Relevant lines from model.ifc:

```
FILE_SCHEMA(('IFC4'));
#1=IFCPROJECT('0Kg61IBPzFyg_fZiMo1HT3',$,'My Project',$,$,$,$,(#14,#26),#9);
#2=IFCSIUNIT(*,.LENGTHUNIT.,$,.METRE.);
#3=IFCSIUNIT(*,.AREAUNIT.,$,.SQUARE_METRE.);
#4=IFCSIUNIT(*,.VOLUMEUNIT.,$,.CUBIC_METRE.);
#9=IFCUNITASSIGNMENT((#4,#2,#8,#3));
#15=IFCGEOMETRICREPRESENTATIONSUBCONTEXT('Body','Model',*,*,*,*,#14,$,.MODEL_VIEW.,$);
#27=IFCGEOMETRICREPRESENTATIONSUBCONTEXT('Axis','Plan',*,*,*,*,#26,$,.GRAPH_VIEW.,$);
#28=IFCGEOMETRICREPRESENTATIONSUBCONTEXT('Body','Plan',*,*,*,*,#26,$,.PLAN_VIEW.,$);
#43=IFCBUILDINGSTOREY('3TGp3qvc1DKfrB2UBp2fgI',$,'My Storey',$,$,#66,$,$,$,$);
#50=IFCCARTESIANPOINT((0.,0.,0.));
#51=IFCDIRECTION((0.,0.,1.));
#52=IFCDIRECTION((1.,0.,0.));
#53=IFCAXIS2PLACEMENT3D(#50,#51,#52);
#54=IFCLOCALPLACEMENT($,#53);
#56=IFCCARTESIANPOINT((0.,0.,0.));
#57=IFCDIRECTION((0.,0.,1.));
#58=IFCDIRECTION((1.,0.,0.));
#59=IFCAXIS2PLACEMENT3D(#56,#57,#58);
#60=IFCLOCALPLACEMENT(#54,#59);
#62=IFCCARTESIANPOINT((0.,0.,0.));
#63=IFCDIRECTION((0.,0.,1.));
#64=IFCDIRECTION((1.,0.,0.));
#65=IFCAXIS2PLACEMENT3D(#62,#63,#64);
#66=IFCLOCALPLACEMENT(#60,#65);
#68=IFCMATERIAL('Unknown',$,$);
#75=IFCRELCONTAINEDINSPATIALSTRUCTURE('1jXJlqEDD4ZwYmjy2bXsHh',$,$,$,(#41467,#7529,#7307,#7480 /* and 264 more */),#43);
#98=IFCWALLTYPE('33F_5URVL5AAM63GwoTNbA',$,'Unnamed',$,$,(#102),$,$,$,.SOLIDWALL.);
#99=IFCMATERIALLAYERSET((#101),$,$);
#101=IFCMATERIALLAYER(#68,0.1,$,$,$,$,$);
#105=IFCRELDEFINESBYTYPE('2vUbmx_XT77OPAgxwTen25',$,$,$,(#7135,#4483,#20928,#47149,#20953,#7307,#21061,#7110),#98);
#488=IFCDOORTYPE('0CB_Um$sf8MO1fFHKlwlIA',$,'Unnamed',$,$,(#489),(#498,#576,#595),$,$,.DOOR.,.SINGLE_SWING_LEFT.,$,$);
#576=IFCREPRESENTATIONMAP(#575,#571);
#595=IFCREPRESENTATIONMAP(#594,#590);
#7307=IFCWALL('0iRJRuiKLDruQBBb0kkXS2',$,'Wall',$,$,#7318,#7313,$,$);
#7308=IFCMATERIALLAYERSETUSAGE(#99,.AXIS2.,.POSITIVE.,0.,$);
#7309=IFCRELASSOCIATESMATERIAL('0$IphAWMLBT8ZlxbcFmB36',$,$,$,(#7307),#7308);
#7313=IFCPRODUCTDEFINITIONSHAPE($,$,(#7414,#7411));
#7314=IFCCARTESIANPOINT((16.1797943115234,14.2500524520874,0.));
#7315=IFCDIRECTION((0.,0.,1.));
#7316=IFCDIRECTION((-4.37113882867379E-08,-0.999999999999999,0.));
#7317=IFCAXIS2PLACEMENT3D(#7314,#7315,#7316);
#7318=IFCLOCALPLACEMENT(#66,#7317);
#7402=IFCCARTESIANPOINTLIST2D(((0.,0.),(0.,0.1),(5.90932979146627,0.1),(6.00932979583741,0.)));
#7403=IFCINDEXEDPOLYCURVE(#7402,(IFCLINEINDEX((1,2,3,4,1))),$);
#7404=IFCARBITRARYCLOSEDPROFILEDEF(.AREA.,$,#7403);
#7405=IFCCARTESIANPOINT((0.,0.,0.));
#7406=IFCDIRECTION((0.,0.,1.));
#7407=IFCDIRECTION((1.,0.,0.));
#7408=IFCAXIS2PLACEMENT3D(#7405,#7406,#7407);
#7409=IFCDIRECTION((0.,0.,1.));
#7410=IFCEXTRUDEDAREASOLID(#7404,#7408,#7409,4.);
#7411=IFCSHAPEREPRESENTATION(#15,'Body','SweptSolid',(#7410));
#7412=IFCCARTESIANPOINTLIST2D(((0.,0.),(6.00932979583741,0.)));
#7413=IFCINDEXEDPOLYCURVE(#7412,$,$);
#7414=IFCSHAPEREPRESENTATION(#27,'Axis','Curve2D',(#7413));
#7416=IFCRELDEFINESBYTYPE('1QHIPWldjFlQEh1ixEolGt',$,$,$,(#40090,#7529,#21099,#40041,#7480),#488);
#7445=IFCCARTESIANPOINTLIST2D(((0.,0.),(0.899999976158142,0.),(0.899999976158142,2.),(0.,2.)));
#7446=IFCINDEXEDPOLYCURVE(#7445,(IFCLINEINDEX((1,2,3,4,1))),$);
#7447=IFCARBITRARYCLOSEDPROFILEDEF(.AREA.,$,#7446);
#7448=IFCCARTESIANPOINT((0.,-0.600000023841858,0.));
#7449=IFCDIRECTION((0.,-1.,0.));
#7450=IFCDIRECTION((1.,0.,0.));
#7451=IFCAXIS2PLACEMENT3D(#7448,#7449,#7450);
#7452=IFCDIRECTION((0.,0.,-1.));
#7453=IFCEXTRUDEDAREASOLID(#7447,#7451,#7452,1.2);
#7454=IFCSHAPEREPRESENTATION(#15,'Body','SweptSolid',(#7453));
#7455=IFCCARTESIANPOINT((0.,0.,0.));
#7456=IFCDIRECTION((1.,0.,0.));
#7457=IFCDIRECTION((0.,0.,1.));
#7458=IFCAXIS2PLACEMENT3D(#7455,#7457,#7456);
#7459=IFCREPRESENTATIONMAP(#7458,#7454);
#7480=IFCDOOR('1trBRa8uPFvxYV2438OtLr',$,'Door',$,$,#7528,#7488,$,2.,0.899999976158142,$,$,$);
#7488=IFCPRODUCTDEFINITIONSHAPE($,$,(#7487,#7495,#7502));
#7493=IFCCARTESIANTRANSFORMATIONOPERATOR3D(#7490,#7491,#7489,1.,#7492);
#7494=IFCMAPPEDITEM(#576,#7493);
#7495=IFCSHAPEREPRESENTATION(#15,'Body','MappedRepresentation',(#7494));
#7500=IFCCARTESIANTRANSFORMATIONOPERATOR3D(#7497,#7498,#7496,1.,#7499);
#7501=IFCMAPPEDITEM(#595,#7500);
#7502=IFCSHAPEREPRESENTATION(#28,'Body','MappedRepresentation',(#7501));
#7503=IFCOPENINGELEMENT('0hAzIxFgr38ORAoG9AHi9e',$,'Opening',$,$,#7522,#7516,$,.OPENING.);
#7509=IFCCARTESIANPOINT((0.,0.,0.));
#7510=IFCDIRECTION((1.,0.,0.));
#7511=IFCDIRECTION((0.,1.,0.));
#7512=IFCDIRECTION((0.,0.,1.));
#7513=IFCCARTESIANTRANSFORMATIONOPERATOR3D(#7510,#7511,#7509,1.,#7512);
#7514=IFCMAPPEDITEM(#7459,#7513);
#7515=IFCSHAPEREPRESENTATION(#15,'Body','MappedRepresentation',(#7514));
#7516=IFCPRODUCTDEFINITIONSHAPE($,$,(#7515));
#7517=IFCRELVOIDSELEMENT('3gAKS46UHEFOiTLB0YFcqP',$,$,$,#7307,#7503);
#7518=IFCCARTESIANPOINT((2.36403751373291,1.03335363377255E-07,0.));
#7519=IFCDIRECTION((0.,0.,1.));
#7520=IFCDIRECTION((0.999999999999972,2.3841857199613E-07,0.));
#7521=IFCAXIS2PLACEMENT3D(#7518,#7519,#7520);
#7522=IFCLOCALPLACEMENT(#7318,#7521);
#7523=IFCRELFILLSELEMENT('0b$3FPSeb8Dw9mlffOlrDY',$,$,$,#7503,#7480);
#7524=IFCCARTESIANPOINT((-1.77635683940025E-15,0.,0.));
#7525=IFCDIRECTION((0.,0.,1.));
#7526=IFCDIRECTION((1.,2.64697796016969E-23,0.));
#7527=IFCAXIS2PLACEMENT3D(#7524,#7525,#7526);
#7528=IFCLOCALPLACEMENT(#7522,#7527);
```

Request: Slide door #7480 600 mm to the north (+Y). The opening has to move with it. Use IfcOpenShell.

```python
import ifcopenshell
import ifcopenshell.api.geometry
import ifcopenshell.util.placement

model = ifcopenshell.open("model.ifc")

door = model.by_id(7480)
opening = door.FillsVoids[0].RelatingOpeningElement
wall = opening.VoidsElements[0].RelatingBuildingElement

wall_matrix = ifcopenshell.util.placement.get_local_placement(wall.ObjectPlacement)
shift = wall_matrix[:3, 0] * -0.6
before = ifcopenshell.util.placement.get_local_placement(door.ObjectPlacement)[:3, 3].copy()

# The door is placed relative to its opening, so it follows when the opening moves.
matrix = ifcopenshell.util.placement.get_local_placement(opening.ObjectPlacement)
matrix[:3, 3] += shift
ifcopenshell.api.geometry.edit_object_placement(
    model, product=opening, matrix=matrix, is_si=False, should_transform_children=True
)

after = ifcopenshell.util.placement.get_local_placement(door.ObjectPlacement)[:3, 3]
print("door moved by", (after - before).round(3) + 0.0)

model.write("model_rev.ifc")
```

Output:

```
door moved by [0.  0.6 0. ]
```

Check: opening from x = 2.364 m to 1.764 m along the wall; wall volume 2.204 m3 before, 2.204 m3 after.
